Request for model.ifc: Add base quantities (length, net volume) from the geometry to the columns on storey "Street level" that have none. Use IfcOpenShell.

First a look at what the model holds.

```python
import ifcopenshell
import ifcopenshell.util.element
import ifcopenshell.util.unit

model = ifcopenshell.open("model.ifc")
print(model.schema)
for unit_type in ("LENGTHUNIT", "AREAUNIT", "VOLUMEUNIT"):
    print(unit_type, ifcopenshell.util.unit.calculate_unit_scale(model, unit_type))
storey = next(s for s in model.by_type("IfcBuildingStorey") if s.Name == "Street level")
columns = [e for e in ifcopenshell.util.element.get_decomposition(storey) if e.is_a("IfcColumn")]
for e in sorted(columns, key=lambda e: e.id()):
    print(e.id(), e.is_a(), e.Name, list(ifcopenshell.util.element.get_psets(e, qtos_only=True)), sep=" | ")
```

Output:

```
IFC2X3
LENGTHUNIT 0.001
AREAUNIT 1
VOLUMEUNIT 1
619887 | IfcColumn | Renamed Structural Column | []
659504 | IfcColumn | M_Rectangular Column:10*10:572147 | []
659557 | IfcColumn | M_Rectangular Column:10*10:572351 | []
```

```python
import ifcopenshell
import ifcopenshell.api.pset
import ifcopenshell.geom
import ifcopenshell.util.element
import ifcopenshell.util.shape
import ifcopenshell.util.unit

model = ifcopenshell.open("model.ifc")
unit_scale = ifcopenshell.util.unit.calculate_unit_scale(model)
volume_scale = ifcopenshell.util.unit.calculate_unit_scale(model, "VOLUMEUNIT")
settings = ifcopenshell.geom.settings()

storey = next(s for s in model.by_type("IfcBuildingStorey") if s.Name == "Street level")
columns = [e for e in ifcopenshell.util.element.get_decomposition(storey) if e.is_a("IfcColumn")]

for e in sorted(columns, key=lambda e: e.id()):
    if ifcopenshell.util.element.get_psets(e, qtos_only=True, should_inherit=False):
        continue
    # Geometry comes back in metres, in the element's own axes.
    shape = ifcopenshell.geom.create_shape(settings, e)
    values = {
        "Length": ifcopenshell.util.shape.get_z(shape.geometry) / unit_scale,
        "NetVolume": ifcopenshell.util.shape.get_volume(shape.geometry) / volume_scale,
    }
    qto = ifcopenshell.api.pset.add_qto(model, product=e, name="BaseQuantities")
    ifcopenshell.api.pset.edit_qto(model, qto=qto, properties=values)
    print(e.id(), {k: round(v, 3) for k, v in values.items()})

model.write("model_updated.ifc")
```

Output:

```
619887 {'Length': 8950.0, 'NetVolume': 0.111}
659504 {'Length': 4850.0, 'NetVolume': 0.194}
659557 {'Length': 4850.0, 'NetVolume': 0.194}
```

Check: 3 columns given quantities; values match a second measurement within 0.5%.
